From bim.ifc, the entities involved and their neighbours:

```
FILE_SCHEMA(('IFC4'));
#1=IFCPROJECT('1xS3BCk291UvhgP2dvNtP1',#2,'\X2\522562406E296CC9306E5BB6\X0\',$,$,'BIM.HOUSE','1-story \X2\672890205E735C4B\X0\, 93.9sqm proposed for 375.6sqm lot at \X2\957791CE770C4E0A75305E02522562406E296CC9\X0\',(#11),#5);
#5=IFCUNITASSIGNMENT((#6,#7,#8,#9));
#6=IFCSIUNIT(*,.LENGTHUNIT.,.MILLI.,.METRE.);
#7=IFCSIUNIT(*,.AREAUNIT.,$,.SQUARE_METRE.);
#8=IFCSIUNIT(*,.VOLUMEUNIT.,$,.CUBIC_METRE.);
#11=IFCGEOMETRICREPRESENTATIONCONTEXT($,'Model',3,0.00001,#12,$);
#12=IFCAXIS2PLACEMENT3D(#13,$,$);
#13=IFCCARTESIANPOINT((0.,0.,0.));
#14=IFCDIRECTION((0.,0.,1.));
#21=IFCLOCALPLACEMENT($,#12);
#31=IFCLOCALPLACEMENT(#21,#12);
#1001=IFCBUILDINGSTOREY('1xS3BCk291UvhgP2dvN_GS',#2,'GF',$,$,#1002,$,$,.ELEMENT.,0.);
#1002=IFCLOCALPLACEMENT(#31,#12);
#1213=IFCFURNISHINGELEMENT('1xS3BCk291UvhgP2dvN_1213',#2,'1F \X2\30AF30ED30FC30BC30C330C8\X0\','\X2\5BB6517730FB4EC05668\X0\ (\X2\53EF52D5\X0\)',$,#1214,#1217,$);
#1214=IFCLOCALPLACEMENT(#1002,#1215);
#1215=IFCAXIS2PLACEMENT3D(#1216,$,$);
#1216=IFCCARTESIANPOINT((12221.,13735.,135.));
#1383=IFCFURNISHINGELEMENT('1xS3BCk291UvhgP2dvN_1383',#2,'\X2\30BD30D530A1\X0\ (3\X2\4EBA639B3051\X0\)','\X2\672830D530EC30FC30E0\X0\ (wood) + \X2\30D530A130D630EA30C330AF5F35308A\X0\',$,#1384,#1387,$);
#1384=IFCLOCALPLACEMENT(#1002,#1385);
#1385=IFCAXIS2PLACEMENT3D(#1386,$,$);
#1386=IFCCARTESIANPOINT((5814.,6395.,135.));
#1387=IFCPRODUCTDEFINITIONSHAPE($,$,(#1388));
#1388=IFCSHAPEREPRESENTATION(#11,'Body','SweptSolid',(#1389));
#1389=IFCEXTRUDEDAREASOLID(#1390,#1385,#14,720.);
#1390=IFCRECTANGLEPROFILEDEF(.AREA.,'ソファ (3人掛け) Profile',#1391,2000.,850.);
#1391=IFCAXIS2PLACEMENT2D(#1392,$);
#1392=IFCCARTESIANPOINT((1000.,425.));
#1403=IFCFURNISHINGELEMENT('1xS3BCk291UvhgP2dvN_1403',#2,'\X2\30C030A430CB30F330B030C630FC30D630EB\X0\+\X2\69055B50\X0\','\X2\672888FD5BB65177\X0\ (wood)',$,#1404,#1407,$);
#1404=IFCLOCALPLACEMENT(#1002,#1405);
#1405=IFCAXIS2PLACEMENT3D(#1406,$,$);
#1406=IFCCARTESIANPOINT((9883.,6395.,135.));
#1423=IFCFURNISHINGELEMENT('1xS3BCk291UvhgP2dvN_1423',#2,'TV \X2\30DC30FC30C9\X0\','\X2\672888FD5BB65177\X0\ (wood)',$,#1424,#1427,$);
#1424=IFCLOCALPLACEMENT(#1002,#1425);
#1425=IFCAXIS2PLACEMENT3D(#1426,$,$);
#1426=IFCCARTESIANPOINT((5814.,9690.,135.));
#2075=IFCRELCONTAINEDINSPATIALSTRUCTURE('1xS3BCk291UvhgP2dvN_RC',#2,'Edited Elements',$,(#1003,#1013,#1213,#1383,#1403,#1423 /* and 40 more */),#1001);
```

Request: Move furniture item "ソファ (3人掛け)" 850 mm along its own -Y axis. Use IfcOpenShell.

```python
import ifcopenshell
import ifcopenshell.api.geometry
import ifcopenshell.util.placement
import ifcopenshell.util.unit

model = ifcopenshell.open("bim.ifc")
unit_scale = ifcopenshell.util.unit.calculate_unit_scale(model)

item = model.by_guid("1xS3BCk291UvhgP2dvN_1383")
matrix = ifcopenshell.util.placement.get_local_placement(item.ObjectPlacement)
matrix[:3, 3] -= matrix[:3, 1] * 0.85 / unit_scale
ifcopenshell.api.geometry.edit_object_placement(model, product=item, matrix=matrix, is_si=False)

print(ifcopenshell.util.placement.get_local_placement(item.ObjectPlacement).round(3) + 0.0)

model.write("bim_v2.ifc")
```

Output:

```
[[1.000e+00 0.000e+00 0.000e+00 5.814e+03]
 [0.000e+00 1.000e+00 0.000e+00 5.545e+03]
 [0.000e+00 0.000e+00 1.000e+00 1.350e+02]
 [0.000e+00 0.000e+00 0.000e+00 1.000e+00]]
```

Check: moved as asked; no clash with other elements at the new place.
